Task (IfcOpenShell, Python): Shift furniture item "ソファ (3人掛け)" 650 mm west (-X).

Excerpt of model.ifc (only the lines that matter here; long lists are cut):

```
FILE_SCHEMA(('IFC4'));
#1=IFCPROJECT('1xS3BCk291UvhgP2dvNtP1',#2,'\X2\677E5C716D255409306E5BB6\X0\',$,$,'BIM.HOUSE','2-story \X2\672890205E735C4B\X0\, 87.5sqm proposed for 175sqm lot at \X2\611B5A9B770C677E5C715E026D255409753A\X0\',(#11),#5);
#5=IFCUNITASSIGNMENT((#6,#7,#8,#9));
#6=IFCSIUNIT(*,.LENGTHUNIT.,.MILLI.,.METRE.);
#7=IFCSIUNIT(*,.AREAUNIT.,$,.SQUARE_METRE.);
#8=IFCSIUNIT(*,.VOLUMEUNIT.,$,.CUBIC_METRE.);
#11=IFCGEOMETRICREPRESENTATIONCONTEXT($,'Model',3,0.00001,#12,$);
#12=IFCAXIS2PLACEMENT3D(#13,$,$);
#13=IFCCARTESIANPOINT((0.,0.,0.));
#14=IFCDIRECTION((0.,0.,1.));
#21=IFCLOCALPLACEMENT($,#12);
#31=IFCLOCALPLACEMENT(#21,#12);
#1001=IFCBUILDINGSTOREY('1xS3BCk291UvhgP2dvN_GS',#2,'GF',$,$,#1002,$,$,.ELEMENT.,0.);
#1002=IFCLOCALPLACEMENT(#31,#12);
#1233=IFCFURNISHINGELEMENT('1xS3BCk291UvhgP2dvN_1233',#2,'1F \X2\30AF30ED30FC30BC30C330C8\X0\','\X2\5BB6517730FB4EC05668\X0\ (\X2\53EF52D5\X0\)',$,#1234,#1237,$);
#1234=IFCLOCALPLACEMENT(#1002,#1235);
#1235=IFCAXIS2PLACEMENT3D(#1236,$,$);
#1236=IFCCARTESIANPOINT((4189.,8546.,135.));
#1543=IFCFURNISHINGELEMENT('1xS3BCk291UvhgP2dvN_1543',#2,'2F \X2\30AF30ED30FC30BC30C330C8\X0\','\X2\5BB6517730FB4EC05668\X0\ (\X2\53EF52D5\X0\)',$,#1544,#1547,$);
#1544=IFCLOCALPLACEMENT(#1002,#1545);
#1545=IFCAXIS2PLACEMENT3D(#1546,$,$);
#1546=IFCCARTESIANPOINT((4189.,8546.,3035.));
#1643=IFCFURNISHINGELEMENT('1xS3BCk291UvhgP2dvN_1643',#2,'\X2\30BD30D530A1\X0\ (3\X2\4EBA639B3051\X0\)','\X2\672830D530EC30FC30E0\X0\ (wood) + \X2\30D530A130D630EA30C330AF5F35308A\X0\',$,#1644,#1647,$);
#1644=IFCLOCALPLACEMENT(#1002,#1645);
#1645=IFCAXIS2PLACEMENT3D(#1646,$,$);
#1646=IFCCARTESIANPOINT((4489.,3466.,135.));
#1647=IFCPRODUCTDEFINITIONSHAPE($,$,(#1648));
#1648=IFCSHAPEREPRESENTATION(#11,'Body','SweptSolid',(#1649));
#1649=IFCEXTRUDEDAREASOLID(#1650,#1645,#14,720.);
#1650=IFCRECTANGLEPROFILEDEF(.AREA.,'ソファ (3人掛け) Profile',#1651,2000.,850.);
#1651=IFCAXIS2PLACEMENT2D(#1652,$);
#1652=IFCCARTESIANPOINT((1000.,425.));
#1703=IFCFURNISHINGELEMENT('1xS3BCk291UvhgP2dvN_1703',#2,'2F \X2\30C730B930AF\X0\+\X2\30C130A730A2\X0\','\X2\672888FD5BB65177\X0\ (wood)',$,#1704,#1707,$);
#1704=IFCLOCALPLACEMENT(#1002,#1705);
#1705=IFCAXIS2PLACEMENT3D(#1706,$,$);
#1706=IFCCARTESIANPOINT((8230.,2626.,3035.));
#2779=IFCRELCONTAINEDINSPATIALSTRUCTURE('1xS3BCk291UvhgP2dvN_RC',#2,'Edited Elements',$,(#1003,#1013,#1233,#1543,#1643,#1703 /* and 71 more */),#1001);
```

```python
import ifcopenshell
import ifcopenshell.api.geometry
import ifcopenshell.util.placement
import ifcopenshell.util.unit

model = ifcopenshell.open("model.ifc")
unit_scale = ifcopenshell.util.unit.calculate_unit_scale(model)

item = model.by_id(1643)
matrix = ifcopenshell.util.placement.get_local_placement(item.ObjectPlacement)
matrix[0, 3] -= 0.65 / unit_scale
ifcopenshell.api.geometry.edit_object_placement(model, product=item, matrix=matrix, is_si=False)

print(ifcopenshell.util.placement.get_local_placement(item.ObjectPlacement).round(3) + 0.0)

model.write("model_edited.ifc")
```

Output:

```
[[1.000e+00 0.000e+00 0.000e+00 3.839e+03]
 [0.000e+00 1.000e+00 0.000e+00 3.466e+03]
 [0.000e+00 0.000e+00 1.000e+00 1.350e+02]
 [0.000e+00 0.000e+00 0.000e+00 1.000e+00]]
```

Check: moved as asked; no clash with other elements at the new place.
